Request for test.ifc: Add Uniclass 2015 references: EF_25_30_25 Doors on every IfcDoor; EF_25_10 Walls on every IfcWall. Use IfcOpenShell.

First a look at what the model holds.

```python
import ifcopenshell

model = ifcopenshell.open("test.ifc")
print(model.schema)
print("classifications:", [c.Name for c in model.by_type("IfcClassification")])
for ifc_class in ("IfcDoor", "IfcRoof", "IfcStair", "IfcWall", "IfcWindow"):
    print(ifc_class, len(model.by_type(ifc_class)))
```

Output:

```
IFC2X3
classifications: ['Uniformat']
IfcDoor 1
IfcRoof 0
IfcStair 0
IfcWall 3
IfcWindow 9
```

```python
import ifcopenshell
import ifcopenshell.api.classification

model = ifcopenshell.open("test.ifc")

# IFC2X3 requires Source and Edition and has no link from the project to the system.
system = model.create_entity("IfcClassification", Source="NBS", Edition="2015", Name="Uniclass 2015")

codes = {
    "IfcDoor": ("EF_25_30_25", "Doors"),
    "IfcWall": ("EF_25_10", "Walls"),
}
for ifc_class, (code, name) in codes.items():
    products = model.by_type(ifc_class)
    ifcopenshell.api.classification.add_reference(
        model, products=products, classification=system, identification=code, name=name
    )
    print(code, len(products))

model.write("test-out.ifc")
```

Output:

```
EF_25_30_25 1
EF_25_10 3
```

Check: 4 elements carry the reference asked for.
